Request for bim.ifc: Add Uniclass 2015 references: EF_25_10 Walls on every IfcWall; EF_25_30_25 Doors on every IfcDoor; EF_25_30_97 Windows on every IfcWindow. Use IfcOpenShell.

First a look at what the model holds.

```python
import ifcopenshell

model = ifcopenshell.open("bim.ifc")
print(model.schema)
print("classifications:", [c.Name for c in model.by_type("IfcClassification")])
for ifc_class in ("IfcDoor", "IfcRoof", "IfcStair", "IfcWall", "IfcWindow"):
    print(ifc_class, len(model.by_type(ifc_class)))
```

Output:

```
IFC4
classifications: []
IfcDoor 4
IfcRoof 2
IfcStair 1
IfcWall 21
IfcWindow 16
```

```python
import ifcopenshell
import ifcopenshell.api.classification

model = ifcopenshell.open("bim.ifc")

system = ifcopenshell.api.classification.add_classification(model, classification="Uniclass 2015")

codes = {
    "IfcWall": ("EF_25_10", "Walls"),
    "IfcDoor": ("EF_25_30_25", "Doors"),
    "IfcWindow": ("EF_25_30_97", "Windows"),
}
for ifc_class, (code, name) in codes.items():
    products = model.by_type(ifc_class)
    ifcopenshell.api.classification.add_reference(
        model, products=products, classification=system, identification=code, name=name
    )
    print(code, len(products))

model.write("bim_v2.ifc")
```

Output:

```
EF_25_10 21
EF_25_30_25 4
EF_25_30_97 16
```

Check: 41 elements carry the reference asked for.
